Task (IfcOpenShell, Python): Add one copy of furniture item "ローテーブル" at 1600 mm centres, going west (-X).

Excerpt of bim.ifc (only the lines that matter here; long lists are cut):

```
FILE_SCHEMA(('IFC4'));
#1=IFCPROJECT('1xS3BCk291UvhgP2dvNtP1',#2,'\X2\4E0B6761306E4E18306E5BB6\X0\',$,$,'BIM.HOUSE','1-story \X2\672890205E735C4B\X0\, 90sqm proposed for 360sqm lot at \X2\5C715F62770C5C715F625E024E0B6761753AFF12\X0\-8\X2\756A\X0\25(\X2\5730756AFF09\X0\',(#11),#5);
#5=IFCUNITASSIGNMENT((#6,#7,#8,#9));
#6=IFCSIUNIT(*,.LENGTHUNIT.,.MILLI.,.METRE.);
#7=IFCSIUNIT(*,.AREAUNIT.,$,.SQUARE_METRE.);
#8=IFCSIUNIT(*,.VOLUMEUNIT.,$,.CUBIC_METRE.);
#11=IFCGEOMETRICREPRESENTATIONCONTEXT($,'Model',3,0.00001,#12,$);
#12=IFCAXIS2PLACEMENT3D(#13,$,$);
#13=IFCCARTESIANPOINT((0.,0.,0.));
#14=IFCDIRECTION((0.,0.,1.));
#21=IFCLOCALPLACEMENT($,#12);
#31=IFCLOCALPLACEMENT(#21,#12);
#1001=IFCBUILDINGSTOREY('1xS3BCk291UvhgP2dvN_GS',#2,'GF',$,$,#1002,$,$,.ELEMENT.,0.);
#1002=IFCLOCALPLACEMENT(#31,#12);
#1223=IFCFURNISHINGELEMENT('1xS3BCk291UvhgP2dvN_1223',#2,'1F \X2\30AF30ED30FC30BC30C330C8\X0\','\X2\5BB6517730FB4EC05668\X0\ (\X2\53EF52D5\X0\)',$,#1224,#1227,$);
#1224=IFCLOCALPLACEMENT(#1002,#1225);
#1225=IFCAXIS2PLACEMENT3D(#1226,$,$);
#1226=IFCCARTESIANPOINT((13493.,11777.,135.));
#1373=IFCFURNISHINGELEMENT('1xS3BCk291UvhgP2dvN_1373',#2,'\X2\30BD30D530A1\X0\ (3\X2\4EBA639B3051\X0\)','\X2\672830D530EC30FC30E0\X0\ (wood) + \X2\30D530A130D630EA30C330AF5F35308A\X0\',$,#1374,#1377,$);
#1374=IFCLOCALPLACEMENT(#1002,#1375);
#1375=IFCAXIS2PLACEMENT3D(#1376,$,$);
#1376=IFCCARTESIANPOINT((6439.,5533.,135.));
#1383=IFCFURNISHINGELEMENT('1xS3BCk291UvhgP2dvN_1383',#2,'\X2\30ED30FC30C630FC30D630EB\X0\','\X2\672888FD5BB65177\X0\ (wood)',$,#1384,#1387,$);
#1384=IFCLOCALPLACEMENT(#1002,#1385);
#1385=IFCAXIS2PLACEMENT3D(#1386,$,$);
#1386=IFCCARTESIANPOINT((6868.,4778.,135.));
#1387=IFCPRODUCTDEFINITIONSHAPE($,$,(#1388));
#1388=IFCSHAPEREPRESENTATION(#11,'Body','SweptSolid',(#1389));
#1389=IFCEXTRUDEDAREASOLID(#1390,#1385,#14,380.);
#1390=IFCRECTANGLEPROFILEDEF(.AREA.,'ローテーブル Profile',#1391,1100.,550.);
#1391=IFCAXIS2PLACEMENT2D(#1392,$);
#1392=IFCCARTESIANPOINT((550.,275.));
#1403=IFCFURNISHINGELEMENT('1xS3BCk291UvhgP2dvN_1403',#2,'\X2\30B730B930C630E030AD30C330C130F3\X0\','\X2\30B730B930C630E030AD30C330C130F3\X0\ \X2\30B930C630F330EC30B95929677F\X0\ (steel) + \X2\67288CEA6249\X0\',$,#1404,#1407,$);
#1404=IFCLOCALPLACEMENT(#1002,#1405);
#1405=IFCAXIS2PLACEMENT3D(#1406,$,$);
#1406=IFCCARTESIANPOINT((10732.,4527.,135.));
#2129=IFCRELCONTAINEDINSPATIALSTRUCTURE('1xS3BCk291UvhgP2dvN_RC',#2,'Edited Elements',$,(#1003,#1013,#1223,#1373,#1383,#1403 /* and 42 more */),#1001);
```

```python
import numpy as np
import ifcopenshell
import ifcopenshell.api.geometry
import ifcopenshell.api.root
import ifcopenshell.util.element
import ifcopenshell.util.placement

model = ifcopenshell.open("bim.ifc")


def reuse_history(source, copy):
    """copy_class also copies each property set's owner history, people and application; keep the originals."""
    for rel in copy.IsDefinedBy:
        if rel.is_a("IfcRelDefinesByProperties") and (history := rel.RelatingPropertyDefinition.OwnerHistory):
            rel.RelatingPropertyDefinition.OwnerHistory = source.OwnerHistory
            ifcopenshell.util.element.remove_deep2(model, history)


source = model.by_guid("1xS3BCk291UvhgP2dvN_1383")
base = ifcopenshell.util.placement.get_local_placement(source.ObjectPlacement)
step = np.array([-1.0, 0.0, 0.0]) * 1600.0

for i in range(1, 2):
    copy = ifcopenshell.api.root.copy_class(model, product=source)
    copy.Representation = ifcopenshell.util.element.copy_deep(
        model, source.Representation, exclude=["IfcGeometricRepresentationContext", "IfcRepresentationMap"]
    )
    reuse_history(source, copy)
    matrix = base.copy()
    matrix[:3, 3] += i * step
    print("added at", matrix[:3, 3].round(3) + 0.0)
    ifcopenshell.api.geometry.edit_object_placement(model, product=copy, matrix=matrix, is_si=False)

model.write("bim-out.ifc")
```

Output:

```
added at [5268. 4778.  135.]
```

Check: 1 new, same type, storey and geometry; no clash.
